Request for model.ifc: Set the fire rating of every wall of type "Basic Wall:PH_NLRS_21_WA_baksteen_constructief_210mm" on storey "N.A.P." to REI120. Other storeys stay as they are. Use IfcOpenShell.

First a look at what the model holds.

```python
import ifcopenshell
import ifcopenshell.util.element

model = ifcopenshell.open("model.ifc")
print(model.schema)
storey = next(s for s in model.by_type("IfcBuildingStorey") if s.Name == "N.A.P.")
walls = [e for e in ifcopenshell.util.element.get_decomposition(storey) if e.is_a("IfcWall")]
seen = {}
for e in walls:
    element_type = ifcopenshell.util.element.get_type(e)
    key = (element_type.Name if element_type != e and element_type else None, ifcopenshell.util.element.get_pset(e, "Pset_WallCommon", "FireRating"))
    seen[key] = seen.get(key, 0) + 1
for (name, value), count in sorted(seen.items(), key=str):
    print(count, "x", name, "|", value)
```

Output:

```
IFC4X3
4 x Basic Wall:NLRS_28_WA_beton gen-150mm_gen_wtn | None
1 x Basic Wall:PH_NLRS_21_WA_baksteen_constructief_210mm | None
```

```python
import ifcopenshell
import ifcopenshell.api.pset
import ifcopenshell.util.element

model = ifcopenshell.open("model.ifc")

storey = next(s for s in model.by_type("IfcBuildingStorey") if s.Name == "N.A.P.")
walls = [e for e in ifcopenshell.util.element.get_decomposition(storey) if e.is_a("IfcWall")]

count = 0
for e in walls:
    element_type = ifcopenshell.util.element.get_type(e)
    if element_type in (None, e) or element_type.Name != "Basic Wall:PH_NLRS_21_WA_baksteen_constructief_210mm":
        continue
    # add_pset returns the element's existing set when there is one.
    pset = ifcopenshell.api.pset.add_pset(model, product=e, name="Pset_WallCommon")
    ifcopenshell.api.pset.edit_pset(model, pset=pset, properties={"FireRating": "REI120"})
    count += 1

print(count, "walls updated")

model.write("model_v2.ifc")
```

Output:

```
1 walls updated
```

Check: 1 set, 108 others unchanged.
